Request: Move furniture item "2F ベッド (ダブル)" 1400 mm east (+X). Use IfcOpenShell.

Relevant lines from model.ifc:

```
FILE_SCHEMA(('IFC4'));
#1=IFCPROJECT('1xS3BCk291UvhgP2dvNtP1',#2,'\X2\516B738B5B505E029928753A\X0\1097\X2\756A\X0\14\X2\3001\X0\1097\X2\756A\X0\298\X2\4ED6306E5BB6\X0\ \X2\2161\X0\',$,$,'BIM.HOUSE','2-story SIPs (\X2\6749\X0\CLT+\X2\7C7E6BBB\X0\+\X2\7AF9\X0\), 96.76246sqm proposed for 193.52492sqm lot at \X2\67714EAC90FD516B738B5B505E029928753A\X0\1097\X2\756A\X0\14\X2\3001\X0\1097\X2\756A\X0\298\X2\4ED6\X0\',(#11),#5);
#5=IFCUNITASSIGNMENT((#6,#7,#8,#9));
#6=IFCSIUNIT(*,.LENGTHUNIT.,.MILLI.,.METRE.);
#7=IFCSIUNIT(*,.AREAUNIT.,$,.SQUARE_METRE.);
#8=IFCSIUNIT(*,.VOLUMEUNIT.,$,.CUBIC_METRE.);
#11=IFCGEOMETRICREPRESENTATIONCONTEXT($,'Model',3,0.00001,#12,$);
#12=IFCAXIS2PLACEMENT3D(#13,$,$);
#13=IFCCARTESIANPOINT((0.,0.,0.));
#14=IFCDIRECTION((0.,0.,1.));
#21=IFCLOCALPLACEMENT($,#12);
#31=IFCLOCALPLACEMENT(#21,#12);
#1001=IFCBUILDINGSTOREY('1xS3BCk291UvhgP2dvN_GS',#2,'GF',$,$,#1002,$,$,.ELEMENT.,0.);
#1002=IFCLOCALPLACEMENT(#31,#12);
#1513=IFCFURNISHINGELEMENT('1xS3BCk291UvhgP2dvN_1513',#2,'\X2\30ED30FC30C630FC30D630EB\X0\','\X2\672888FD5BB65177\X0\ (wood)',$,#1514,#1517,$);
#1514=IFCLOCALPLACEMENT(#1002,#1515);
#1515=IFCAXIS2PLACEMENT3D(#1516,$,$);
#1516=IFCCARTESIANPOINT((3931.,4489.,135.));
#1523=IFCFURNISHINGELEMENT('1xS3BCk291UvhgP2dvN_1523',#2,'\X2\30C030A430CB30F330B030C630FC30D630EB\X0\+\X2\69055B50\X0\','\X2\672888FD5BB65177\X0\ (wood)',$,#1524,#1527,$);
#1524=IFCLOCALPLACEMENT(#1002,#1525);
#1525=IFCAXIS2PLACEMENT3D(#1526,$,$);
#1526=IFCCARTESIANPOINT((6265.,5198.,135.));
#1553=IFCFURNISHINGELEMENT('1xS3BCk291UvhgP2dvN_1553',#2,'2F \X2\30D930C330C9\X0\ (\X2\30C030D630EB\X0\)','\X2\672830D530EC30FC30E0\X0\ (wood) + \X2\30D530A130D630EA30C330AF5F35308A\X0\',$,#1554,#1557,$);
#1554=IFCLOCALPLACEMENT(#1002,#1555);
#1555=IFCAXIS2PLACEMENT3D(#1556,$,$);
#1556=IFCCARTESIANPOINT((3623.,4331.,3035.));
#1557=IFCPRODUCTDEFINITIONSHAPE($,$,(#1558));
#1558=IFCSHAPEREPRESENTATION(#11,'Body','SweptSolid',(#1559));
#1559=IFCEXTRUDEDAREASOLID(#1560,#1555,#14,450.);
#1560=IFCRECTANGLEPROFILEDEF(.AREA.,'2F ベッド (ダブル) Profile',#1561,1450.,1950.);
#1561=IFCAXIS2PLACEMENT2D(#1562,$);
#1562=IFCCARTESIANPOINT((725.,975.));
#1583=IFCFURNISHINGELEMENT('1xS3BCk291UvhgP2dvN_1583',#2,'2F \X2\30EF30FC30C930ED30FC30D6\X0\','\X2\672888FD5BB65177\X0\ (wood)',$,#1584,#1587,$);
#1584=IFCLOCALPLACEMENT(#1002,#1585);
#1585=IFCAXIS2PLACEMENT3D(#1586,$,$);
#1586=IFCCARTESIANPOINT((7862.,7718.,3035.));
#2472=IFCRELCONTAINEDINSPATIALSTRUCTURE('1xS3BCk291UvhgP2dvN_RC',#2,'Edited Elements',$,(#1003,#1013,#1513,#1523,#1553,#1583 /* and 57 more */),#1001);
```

```python
import ifcopenshell
import ifcopenshell.api.geometry
import ifcopenshell.util.placement
import ifcopenshell.util.unit

model = ifcopenshell.open("model.ifc")
unit_scale = ifcopenshell.util.unit.calculate_unit_scale(model)

item = model.by_id(1553)
matrix = ifcopenshell.util.placement.get_local_placement(item.ObjectPlacement)
matrix[0, 3] += 1.4 / unit_scale
ifcopenshell.api.geometry.edit_object_placement(model, product=item, matrix=matrix, is_si=False)

print(ifcopenshell.util.placement.get_local_placement(item.ObjectPlacement).round(3) + 0.0)

model.write("model_updated.ifc")
```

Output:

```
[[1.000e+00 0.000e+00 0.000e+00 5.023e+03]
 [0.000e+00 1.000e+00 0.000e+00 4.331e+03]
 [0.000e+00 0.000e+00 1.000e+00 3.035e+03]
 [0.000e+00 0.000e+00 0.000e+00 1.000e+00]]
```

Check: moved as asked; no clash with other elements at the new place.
